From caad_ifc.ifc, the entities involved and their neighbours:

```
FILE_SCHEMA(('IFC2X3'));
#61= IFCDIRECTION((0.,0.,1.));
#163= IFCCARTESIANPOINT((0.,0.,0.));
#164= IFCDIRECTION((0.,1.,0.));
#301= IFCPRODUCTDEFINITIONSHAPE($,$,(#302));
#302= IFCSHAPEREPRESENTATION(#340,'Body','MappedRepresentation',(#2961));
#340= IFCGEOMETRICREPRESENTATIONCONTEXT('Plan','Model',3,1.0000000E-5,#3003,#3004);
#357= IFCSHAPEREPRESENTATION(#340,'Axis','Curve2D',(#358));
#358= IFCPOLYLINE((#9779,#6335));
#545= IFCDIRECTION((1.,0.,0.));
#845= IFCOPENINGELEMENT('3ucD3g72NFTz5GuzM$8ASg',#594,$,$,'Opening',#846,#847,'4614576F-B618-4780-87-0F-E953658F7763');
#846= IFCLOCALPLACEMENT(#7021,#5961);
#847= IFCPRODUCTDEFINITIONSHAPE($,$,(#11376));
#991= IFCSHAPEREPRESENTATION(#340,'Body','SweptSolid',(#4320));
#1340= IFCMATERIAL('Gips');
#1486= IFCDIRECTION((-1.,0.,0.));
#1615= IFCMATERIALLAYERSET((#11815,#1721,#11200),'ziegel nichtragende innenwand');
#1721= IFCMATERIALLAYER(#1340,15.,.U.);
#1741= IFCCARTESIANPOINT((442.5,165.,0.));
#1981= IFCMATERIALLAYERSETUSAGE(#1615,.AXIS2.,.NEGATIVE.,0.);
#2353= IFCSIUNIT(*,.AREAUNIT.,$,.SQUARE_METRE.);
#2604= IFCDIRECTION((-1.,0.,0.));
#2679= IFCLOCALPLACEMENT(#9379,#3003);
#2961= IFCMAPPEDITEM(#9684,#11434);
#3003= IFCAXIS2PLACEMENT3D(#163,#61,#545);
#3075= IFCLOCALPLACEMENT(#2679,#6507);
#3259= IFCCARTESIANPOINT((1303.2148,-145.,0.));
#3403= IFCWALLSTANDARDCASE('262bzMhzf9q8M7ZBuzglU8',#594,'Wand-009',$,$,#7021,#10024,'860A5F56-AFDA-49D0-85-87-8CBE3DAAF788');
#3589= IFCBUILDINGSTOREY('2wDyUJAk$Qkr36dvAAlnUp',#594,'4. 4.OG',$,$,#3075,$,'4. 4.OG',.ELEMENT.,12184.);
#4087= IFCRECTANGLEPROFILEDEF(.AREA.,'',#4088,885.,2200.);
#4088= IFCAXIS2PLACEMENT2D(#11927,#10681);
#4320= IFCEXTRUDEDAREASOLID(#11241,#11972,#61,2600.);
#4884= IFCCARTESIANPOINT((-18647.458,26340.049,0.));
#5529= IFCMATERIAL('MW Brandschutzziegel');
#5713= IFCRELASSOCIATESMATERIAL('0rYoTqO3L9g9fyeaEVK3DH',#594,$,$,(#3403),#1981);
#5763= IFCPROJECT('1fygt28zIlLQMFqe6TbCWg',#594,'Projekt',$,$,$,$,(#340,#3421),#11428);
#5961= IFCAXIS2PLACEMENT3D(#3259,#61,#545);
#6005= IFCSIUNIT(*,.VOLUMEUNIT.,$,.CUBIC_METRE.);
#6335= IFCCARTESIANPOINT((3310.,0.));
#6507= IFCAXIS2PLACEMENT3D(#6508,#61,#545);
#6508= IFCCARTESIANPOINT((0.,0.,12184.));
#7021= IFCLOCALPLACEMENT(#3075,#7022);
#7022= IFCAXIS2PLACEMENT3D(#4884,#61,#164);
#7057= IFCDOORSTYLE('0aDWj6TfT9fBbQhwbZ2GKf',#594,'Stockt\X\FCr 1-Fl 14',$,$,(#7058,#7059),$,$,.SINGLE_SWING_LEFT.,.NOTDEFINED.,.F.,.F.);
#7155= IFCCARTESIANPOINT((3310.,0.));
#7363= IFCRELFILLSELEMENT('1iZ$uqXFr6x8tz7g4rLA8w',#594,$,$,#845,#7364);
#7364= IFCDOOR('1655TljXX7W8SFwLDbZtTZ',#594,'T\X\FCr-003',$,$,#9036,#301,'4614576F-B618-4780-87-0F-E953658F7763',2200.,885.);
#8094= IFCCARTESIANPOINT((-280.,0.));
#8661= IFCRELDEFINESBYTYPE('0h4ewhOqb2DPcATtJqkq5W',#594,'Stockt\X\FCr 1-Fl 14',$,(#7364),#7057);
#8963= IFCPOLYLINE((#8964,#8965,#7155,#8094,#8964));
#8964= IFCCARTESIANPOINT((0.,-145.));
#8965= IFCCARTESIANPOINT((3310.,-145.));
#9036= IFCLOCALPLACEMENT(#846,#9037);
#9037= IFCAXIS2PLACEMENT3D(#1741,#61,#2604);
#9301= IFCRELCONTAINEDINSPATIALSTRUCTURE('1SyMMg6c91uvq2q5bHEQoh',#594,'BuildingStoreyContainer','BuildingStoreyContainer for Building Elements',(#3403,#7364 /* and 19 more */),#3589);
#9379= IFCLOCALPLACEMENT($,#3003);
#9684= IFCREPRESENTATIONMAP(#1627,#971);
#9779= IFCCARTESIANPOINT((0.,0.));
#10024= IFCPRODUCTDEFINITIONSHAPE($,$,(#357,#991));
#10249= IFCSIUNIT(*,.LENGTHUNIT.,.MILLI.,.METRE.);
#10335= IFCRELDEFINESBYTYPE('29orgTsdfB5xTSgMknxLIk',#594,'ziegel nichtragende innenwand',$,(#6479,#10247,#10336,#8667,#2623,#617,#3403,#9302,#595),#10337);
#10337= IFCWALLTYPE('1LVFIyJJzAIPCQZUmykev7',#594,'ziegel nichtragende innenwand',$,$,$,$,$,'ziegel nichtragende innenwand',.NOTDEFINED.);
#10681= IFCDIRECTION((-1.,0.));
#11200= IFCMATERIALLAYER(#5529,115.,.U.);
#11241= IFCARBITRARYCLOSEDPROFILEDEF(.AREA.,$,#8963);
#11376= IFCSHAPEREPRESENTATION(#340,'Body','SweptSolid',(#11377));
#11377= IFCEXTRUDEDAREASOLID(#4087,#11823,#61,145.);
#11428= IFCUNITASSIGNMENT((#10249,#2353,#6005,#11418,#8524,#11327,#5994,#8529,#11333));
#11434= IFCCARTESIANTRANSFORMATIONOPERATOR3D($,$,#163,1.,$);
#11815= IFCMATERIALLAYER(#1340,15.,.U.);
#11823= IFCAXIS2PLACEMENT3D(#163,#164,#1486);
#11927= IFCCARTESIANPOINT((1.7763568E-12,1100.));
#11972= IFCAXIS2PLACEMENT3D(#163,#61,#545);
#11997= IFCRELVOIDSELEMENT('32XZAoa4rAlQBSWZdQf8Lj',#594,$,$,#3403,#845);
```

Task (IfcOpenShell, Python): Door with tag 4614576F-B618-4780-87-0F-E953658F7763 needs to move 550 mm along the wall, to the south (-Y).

```python
import ifcopenshell
import ifcopenshell.api.geometry
import ifcopenshell.util.placement
import ifcopenshell.util.unit

model = ifcopenshell.open("caad_ifc.ifc")
unit_scale = ifcopenshell.util.unit.calculate_unit_scale(model)

door = model.by_guid("1655TljXX7W8SFwLDbZtTZ")
opening = door.FillsVoids[0].RelatingOpeningElement
wall = opening.VoidsElements[0].RelatingBuildingElement

wall_matrix = ifcopenshell.util.placement.get_local_placement(wall.ObjectPlacement)
shift = wall_matrix[:3, 0] * -0.55 / unit_scale
before = ifcopenshell.util.placement.get_local_placement(door.ObjectPlacement)[:3, 3].copy()

# The door is placed relative to its opening, so it follows when the opening moves.
matrix = ifcopenshell.util.placement.get_local_placement(opening.ObjectPlacement)
matrix[:3, 3] += shift
ifcopenshell.api.geometry.edit_object_placement(
    model, product=opening, matrix=matrix, is_si=False, should_transform_children=True
)

after = ifcopenshell.util.placement.get_local_placement(door.ObjectPlacement)[:3, 3]
print("door moved by", (after - before).round(3) + 0.0)

model.write("caad_ifc_v2.ifc")
```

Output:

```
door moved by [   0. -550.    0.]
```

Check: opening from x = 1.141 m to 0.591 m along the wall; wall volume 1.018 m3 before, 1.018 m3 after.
